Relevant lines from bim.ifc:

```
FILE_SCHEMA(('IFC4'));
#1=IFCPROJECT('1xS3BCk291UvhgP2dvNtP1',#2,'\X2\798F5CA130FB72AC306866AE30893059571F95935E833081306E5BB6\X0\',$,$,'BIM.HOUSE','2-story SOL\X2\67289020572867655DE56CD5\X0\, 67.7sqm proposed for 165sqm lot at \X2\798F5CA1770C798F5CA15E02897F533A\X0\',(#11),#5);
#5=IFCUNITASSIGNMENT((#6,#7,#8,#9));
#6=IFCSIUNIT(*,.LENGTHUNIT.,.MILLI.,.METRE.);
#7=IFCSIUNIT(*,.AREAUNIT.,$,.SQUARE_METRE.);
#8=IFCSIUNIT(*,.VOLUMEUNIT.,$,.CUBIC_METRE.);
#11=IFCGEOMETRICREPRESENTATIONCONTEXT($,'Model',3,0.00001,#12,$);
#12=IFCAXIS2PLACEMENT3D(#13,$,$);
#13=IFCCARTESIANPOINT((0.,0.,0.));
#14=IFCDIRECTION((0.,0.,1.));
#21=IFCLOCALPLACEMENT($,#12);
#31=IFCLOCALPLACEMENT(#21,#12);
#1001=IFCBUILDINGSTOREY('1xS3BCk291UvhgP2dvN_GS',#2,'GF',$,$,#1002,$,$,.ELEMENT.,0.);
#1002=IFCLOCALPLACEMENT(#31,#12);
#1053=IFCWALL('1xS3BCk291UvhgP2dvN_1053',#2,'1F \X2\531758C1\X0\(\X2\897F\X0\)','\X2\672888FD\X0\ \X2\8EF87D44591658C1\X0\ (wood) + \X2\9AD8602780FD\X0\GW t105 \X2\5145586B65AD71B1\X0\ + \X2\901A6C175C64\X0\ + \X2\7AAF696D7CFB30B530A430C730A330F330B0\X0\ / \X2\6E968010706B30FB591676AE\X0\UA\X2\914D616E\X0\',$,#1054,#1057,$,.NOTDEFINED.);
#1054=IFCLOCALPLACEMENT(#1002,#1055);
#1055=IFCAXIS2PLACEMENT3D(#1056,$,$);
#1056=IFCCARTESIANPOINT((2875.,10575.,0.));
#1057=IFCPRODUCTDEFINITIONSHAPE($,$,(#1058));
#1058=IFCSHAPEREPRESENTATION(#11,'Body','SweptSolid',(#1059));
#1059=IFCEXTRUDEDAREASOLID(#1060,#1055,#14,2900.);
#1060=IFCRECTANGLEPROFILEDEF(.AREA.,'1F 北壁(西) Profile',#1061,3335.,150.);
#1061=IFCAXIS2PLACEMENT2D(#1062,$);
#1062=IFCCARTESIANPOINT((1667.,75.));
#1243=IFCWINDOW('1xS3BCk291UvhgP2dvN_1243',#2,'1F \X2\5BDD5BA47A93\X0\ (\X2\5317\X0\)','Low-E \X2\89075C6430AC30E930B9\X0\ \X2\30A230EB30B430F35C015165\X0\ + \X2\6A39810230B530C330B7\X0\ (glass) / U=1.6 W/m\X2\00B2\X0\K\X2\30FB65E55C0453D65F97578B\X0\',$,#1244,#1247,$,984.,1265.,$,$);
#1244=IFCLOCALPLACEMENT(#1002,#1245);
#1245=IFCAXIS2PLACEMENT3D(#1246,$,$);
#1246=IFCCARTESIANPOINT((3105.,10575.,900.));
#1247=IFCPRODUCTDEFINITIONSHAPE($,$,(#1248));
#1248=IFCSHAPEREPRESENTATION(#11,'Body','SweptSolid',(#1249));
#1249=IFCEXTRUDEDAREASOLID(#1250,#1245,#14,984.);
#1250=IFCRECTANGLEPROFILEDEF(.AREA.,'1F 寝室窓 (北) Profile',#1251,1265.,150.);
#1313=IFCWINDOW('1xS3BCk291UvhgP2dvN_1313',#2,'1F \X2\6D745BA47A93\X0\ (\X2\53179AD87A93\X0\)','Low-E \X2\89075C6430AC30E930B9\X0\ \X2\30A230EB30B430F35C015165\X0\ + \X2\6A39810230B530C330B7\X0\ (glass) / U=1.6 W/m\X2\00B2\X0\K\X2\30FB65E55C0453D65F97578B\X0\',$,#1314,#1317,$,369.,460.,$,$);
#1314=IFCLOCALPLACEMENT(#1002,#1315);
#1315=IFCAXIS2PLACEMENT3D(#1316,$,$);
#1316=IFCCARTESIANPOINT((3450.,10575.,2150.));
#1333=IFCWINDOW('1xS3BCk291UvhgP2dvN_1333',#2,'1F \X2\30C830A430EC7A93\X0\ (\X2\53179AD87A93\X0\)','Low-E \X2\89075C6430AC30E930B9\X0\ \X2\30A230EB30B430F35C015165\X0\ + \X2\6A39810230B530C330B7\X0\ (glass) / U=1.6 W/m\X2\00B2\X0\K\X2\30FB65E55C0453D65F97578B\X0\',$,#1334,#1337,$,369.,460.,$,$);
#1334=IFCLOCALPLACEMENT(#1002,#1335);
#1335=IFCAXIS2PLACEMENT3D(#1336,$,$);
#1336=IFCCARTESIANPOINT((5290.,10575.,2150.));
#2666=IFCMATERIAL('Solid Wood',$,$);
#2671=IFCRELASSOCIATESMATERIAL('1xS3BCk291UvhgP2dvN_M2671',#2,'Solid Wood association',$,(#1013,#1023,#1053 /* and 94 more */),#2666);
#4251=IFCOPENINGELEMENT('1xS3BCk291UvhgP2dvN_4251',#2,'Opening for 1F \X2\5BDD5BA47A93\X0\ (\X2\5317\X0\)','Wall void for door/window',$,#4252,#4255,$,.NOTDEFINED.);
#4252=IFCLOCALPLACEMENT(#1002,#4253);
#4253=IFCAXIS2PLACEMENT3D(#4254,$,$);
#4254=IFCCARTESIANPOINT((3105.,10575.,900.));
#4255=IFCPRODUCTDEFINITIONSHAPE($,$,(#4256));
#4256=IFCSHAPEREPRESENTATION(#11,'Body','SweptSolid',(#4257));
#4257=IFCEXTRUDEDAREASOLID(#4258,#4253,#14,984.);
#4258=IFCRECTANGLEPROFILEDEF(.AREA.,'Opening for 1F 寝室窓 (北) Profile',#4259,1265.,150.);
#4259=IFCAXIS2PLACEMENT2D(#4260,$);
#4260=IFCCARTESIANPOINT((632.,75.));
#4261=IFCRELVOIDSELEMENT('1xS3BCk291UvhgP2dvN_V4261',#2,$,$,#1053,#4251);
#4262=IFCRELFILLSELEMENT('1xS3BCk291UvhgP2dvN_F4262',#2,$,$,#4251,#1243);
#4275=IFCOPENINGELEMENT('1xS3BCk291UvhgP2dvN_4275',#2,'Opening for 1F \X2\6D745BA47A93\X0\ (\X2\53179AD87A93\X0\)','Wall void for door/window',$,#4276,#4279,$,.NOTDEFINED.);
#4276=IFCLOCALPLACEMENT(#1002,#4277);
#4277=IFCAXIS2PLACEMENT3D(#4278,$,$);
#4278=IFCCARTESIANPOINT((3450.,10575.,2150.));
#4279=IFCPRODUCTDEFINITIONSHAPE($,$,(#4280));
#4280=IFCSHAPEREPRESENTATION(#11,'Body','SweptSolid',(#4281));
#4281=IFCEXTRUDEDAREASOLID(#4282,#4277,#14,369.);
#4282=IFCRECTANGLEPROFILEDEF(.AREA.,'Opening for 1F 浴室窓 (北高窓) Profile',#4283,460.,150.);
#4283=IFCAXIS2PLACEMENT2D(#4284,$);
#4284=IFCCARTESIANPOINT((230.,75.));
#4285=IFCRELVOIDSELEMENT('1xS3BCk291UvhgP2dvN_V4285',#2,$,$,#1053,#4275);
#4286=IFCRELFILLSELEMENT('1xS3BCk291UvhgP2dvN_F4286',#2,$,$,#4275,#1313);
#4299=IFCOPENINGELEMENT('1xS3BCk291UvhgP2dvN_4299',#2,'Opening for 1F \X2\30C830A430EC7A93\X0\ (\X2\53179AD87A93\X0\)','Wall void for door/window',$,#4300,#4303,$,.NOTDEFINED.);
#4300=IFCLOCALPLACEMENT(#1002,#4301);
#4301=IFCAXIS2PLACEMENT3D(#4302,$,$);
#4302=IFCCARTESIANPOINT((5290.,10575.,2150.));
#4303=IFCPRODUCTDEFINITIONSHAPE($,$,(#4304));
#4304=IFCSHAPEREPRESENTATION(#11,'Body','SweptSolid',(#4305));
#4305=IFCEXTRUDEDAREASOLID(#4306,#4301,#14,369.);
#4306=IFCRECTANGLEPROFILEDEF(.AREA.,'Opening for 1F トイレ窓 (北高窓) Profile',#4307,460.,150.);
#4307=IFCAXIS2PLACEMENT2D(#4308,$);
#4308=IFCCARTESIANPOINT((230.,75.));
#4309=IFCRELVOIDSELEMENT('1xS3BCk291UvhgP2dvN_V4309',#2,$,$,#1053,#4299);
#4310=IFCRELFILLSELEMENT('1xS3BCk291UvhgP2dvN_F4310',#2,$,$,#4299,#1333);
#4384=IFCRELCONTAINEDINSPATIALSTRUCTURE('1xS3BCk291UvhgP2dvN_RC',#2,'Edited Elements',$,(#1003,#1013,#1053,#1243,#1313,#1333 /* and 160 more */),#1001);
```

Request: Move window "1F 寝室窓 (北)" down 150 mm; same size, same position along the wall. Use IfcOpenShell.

```python
import numpy as np
import ifcopenshell
import ifcopenshell.api.geometry
import ifcopenshell.util.placement
import ifcopenshell.util.unit

model = ifcopenshell.open("bim.ifc")
unit_scale = ifcopenshell.util.unit.calculate_unit_scale(model)

window = model.by_guid("1xS3BCk291UvhgP2dvN_1243")
opening = window.FillsVoids[0].RelatingOpeningElement
dz = -0.15 / unit_scale

shift = np.array([0.0, 0.0, dz])
# The window is not placed relative to its opening, so move both.
for product in (opening, window):
    matrix = ifcopenshell.util.placement.get_local_placement(product.ObjectPlacement)
    matrix[:3, 3] += shift
    ifcopenshell.api.geometry.edit_object_placement(model, product=product, matrix=matrix, is_si=False)

print(f"moved by {dz * unit_scale:+.3f} m")

model.write("bim_updated.ifc")
```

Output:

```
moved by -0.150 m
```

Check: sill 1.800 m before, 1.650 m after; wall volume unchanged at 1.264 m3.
